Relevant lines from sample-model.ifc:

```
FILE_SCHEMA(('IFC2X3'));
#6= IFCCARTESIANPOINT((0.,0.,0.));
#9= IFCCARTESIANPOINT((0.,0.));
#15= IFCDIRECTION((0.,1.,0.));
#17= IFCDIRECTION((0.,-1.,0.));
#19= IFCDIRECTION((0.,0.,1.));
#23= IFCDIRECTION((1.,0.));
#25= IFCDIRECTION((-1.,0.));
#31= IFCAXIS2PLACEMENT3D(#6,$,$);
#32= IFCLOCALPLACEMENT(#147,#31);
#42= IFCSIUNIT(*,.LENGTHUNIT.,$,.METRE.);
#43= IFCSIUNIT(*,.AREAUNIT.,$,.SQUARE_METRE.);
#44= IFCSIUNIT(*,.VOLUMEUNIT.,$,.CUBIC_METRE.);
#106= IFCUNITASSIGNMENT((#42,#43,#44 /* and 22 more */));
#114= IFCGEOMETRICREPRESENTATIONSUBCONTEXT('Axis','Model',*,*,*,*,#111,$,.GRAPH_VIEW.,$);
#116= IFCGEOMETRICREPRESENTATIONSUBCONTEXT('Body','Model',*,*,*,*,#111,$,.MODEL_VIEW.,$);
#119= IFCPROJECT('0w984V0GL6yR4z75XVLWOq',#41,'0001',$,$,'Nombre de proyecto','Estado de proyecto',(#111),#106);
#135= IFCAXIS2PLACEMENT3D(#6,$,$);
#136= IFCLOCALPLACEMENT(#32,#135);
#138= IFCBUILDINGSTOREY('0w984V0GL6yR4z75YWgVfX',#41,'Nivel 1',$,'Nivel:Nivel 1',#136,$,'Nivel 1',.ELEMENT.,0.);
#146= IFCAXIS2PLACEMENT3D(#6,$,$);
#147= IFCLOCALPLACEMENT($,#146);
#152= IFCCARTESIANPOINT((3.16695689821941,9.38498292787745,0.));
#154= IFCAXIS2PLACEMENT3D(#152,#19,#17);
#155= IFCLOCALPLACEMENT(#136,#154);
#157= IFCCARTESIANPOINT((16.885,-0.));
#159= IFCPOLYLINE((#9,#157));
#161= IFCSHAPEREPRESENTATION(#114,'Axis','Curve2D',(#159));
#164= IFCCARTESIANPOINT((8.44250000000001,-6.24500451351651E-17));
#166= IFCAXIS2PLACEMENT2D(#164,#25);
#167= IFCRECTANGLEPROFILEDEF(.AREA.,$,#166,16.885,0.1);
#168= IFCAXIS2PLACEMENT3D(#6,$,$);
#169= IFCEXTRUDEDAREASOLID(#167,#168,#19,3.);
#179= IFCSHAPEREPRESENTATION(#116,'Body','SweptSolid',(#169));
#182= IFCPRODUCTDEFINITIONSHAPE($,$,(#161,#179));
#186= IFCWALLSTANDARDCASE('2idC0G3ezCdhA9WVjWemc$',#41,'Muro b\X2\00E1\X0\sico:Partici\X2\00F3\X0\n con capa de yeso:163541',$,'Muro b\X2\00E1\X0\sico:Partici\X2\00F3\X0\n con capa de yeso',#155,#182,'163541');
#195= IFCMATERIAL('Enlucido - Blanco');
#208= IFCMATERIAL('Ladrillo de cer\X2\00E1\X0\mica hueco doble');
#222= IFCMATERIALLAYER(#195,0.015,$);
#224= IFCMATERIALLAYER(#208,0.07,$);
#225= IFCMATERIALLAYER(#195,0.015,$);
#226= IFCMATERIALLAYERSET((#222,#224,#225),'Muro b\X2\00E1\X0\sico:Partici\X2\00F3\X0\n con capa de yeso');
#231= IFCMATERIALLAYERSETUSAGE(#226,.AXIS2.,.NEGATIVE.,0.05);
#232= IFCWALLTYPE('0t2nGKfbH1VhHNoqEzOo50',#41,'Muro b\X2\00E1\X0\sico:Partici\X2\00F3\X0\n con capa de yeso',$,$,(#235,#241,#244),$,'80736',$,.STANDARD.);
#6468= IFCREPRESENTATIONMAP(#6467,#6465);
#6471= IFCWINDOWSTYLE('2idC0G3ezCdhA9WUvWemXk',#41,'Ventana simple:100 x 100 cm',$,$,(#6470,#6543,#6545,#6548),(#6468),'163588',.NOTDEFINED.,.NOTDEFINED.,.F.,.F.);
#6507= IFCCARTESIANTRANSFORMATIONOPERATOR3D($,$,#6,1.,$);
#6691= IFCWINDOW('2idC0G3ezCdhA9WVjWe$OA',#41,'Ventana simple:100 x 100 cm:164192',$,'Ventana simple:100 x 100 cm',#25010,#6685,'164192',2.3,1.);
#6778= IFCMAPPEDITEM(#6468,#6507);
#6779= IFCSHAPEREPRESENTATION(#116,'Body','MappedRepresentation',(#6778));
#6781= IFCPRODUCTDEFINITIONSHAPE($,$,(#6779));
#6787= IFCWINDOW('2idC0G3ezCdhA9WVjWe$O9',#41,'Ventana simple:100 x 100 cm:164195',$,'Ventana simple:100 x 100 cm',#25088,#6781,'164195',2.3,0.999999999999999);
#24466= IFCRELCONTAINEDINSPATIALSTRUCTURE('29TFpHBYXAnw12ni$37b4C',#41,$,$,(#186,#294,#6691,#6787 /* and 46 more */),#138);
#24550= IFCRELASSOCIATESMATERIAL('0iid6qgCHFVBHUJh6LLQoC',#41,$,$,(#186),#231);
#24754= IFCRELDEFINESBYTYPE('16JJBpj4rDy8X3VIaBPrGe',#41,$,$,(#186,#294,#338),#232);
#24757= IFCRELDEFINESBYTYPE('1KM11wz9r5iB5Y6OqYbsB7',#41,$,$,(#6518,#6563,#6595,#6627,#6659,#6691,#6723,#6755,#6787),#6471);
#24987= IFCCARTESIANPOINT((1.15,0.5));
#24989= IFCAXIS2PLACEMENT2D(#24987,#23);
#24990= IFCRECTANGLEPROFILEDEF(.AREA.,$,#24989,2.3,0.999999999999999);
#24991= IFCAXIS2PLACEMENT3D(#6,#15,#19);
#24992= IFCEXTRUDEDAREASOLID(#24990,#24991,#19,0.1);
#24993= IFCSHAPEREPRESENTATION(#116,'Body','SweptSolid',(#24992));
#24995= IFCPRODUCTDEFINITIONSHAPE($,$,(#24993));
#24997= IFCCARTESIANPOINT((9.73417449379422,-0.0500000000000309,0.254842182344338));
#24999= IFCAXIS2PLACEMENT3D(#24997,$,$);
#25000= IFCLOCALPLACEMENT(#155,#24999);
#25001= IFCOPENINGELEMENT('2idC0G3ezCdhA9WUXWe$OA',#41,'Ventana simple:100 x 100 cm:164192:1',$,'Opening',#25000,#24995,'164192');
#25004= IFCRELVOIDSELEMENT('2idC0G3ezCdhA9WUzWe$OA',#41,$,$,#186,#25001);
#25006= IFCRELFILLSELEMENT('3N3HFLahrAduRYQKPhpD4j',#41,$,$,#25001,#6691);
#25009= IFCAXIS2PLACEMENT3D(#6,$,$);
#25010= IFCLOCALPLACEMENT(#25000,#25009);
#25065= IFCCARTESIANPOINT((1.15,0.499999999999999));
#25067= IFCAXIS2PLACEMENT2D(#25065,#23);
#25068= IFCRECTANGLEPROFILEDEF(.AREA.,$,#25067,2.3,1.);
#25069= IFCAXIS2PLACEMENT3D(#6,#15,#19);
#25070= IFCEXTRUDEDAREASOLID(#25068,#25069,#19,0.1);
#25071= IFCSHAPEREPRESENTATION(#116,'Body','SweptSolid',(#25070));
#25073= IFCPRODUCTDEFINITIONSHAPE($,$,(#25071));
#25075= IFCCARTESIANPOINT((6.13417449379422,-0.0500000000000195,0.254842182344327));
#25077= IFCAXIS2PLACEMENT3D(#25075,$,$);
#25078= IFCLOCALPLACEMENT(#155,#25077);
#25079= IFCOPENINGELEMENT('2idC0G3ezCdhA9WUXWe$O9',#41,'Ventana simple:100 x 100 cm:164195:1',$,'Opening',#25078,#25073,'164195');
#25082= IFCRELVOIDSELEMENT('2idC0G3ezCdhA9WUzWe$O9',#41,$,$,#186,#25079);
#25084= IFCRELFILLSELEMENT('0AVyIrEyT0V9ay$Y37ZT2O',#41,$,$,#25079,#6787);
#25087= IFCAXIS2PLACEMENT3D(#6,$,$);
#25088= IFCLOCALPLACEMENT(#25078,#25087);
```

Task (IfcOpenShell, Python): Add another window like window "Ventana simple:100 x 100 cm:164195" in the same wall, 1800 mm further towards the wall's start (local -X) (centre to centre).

```python
import ifcopenshell
import ifcopenshell.api.feature
import ifcopenshell.api.geometry
import ifcopenshell.api.root
import ifcopenshell.geom
import ifcopenshell.util.element
import ifcopenshell.util.placement
import ifcopenshell.util.shape

model = ifcopenshell.open("sample-model.ifc")
settings = ifcopenshell.geom.settings()


def volume(element):
    """Net volume in cubic metres, openings subtracted."""
    shape = ifcopenshell.geom.create_shape(settings, element)
    return ifcopenshell.util.shape.get_volume(shape.geometry)


def reuse_history(source, copy):
    """copy_class also copies each property set's owner history, people and application; keep the originals."""
    for rel in copy.IsDefinedBy:
        if rel.is_a("IfcRelDefinesByProperties") and (history := rel.RelatingPropertyDefinition.OwnerHistory):
            rel.RelatingPropertyDefinition.OwnerHistory = source.OwnerHistory
            ifcopenshell.util.element.remove_deep2(model, history)


window = model.by_guid("2idC0G3ezCdhA9WVjWe$O9")
opening = window.FillsVoids[0].RelatingOpeningElement
wall = opening.VoidsElements[0].RelatingBuildingElement
before = volume(wall)
shift = ifcopenshell.util.placement.get_local_placement(wall.ObjectPlacement)[:3, 0] * -1.8

# copy_class copies the void relationship, type, container and properties, but no geometry.
new_opening = ifcopenshell.api.root.copy_class(model, product=opening)
new_opening.Representation = ifcopenshell.util.element.copy_deep(
    model, opening.Representation, exclude=["IfcGeometricRepresentationContext", "IfcRepresentationMap"]
)
new_opening.Name = "Ventana simple:100 x 100 cm"
new_opening.Tag = None
new_window = ifcopenshell.api.root.copy_class(model, product=window)
new_window.Representation = ifcopenshell.util.element.copy_deep(
    model, window.Representation, exclude=["IfcGeometricRepresentationContext", "IfcRepresentationMap"]
)
new_window.Name = "Ventana simple:100 x 100 cm"
new_window.Tag = None
reuse_history(window, new_window)
fills = ifcopenshell.api.feature.add_filling(model, opening=new_opening, element=new_window)
fills.OwnerHistory = new_window.OwnerHistory  # required in IFC2X3

for old, new in ((opening, new_opening), (window, new_window)):
    matrix = ifcopenshell.util.placement.get_local_placement(old.ObjectPlacement)
    matrix[:3, 3] += shift
    ifcopenshell.api.geometry.edit_object_placement(model, product=new, matrix=matrix, is_si=False)

after = volume(wall)

print(f"wall volume {before:.3f} -> {after:.3f} m3")

model.write("sample-model_v2.ifc")
```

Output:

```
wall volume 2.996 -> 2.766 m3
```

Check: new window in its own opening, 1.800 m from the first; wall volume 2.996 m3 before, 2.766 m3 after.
